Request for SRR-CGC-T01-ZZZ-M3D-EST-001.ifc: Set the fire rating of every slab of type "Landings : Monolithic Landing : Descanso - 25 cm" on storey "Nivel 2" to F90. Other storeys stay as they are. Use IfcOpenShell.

First a look at what the model holds.

```python
import ifcopenshell
import ifcopenshell.util.element

model = ifcopenshell.open("SRR-CGC-T01-ZZZ-M3D-EST-001.ifc")
print(model.schema)
storey = next(s for s in model.by_type("IfcBuildingStorey") if s.Name == "Nivel 2")
slabs = [e for e in ifcopenshell.util.element.get_decomposition(storey) if e.is_a("IfcSlab")]
seen = {}
for e in slabs:
    element_type = ifcopenshell.util.element.get_type(e)
    key = (element_type.Name if element_type != e and element_type else None, ifcopenshell.util.element.get_pset(e, "Pset_SlabCommon", "FireRating"))
    seen[key] = seen.get(key, 0) + 1
for (name, value), count in sorted(seen.items(), key=str):
    print(count, "x", name, "|", value)
```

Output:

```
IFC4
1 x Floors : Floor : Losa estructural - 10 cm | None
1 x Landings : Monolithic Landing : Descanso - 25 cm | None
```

```python
import ifcopenshell
import ifcopenshell.api.pset
import ifcopenshell.util.element

model = ifcopenshell.open("SRR-CGC-T01-ZZZ-M3D-EST-001.ifc")

storey = next(s for s in model.by_type("IfcBuildingStorey") if s.Name == "Nivel 2")
slabs = [e for e in ifcopenshell.util.element.get_decomposition(storey) if e.is_a("IfcSlab")]

count = 0
for e in slabs:
    element_type = ifcopenshell.util.element.get_type(e)
    if element_type in (None, e) or element_type.Name != "Landings : Monolithic Landing : Descanso - 25 cm":
        continue
    # add_pset returns the element's existing set when there is one.
    pset = ifcopenshell.api.pset.add_pset(model, product=e, name="Pset_SlabCommon")
    ifcopenshell.api.pset.edit_pset(model, pset=pset, properties={"FireRating": "F90"})
    count += 1

print(count, "slabs updated")

model.write("SRR-CGC-T01-ZZZ-M3D-EST-001_v2.ifc")
```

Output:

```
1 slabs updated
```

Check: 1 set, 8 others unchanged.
